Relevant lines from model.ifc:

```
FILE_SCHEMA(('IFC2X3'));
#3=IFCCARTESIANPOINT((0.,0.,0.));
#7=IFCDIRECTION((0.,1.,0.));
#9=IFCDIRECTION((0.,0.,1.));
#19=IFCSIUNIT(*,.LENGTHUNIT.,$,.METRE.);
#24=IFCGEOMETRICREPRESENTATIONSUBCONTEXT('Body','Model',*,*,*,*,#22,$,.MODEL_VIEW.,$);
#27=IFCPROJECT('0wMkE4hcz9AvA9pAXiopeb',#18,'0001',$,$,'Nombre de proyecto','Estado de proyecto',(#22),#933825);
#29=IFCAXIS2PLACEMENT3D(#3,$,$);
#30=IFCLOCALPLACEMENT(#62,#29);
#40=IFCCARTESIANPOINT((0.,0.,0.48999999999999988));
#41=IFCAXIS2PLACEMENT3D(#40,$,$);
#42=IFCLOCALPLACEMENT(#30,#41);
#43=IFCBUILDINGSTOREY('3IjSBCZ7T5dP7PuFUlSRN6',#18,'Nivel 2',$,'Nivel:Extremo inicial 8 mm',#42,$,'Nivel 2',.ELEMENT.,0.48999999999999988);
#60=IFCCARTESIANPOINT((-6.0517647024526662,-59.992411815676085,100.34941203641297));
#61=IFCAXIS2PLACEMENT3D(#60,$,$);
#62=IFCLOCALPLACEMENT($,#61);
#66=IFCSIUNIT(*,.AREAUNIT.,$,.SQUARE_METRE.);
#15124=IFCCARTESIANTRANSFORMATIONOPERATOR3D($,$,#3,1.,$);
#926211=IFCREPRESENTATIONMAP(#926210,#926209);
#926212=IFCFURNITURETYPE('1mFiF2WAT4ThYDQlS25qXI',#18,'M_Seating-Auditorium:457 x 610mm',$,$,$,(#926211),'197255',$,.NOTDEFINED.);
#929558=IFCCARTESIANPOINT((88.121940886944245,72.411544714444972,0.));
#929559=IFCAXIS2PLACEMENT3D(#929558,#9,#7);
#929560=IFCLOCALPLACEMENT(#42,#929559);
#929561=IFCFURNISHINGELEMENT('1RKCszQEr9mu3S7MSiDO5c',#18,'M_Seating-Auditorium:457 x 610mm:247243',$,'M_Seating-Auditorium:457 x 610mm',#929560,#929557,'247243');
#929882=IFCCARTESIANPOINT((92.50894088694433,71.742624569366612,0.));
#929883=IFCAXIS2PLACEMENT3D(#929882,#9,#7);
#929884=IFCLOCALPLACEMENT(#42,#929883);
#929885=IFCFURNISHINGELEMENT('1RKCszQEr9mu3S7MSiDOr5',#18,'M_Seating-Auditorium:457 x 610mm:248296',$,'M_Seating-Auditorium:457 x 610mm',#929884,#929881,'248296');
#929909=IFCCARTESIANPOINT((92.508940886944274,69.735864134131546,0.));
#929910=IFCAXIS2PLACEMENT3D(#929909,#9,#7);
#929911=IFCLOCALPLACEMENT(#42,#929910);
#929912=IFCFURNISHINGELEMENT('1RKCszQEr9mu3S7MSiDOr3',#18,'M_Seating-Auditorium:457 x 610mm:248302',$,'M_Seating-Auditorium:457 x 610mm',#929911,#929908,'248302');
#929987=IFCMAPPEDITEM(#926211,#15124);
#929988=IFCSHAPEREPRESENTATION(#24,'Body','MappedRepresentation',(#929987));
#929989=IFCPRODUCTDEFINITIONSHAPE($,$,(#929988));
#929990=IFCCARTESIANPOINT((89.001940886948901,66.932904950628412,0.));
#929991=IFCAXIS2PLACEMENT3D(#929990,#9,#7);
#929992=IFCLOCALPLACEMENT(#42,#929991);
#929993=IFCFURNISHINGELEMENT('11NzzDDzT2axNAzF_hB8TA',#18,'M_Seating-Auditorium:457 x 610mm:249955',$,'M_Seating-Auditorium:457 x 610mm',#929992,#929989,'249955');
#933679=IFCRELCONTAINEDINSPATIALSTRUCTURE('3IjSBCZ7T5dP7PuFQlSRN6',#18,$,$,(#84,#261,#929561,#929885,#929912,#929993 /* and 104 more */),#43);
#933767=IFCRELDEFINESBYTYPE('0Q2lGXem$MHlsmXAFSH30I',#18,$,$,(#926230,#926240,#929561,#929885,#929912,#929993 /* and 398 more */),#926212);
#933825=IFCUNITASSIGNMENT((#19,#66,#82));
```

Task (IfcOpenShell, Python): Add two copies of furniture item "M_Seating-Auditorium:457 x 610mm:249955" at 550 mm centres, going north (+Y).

```python
import numpy as np
import ifcopenshell
import ifcopenshell.api.geometry
import ifcopenshell.api.root
import ifcopenshell.util.element
import ifcopenshell.util.placement
import ifcopenshell.util.unit

model = ifcopenshell.open("model.ifc")
unit_scale = ifcopenshell.util.unit.calculate_unit_scale(model)


def reuse_history(source, copy):
    """copy_class also copies each property set's owner history, people and application; keep the originals."""
    for rel in copy.IsDefinedBy:
        if rel.is_a("IfcRelDefinesByProperties") and (history := rel.RelatingPropertyDefinition.OwnerHistory):
            rel.RelatingPropertyDefinition.OwnerHistory = source.OwnerHistory
            ifcopenshell.util.element.remove_deep2(model, history)


source = model.by_guid("11NzzDDzT2axNAzF_hB8TA")
base = ifcopenshell.util.placement.get_local_placement(source.ObjectPlacement)
step = np.array([0.0, 1.0, 0.0]) * 0.55 / unit_scale

for i in range(1, 3):
    copy = ifcopenshell.api.root.copy_class(model, product=source)
    copy.Representation = ifcopenshell.util.element.copy_deep(
        model, source.Representation, exclude=["IfcGeometricRepresentationContext", "IfcRepresentationMap"]
    )
    copy.Name = "M_Seating-Auditorium:457 x 610mm"
    copy.Tag = None
    reuse_history(source, copy)
    matrix = base.copy()
    matrix[:3, 3] += i * step
    print("added at", matrix[:3, 3].round(3) + 0.0)
    ifcopenshell.api.geometry.edit_object_placement(model, product=copy, matrix=matrix, is_si=False)

model.write("model_edited.ifc")
```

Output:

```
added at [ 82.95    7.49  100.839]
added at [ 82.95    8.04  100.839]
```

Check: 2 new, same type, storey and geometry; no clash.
